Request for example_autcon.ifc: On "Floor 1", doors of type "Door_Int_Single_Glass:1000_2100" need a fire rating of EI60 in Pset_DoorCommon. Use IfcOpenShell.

First a look at what the model holds.

```python
import ifcopenshell
import ifcopenshell.util.element

model = ifcopenshell.open("example_autcon.ifc")
print(model.schema)
storey = next(s for s in model.by_type("IfcBuildingStorey") if s.Name == "Floor 1")
doors = [e for e in ifcopenshell.util.element.get_decomposition(storey) if e.is_a("IfcDoor")]
seen = {}
for e in doors:
    element_type = ifcopenshell.util.element.get_type(e)
    key = (element_type.Name if element_type != e and element_type else None, ifcopenshell.util.element.get_pset(e, "Pset_DoorCommon", "FireRating"))
    seen[key] = seen.get(key, 0) + 1
for (name, value), count in sorted(seen.items(), key=str):
    print(count, "x", name, "|", value)
```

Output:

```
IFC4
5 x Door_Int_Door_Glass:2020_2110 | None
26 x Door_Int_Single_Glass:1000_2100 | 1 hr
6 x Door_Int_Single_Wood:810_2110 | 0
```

```python
import ifcopenshell
import ifcopenshell.api.pset
import ifcopenshell.util.element

model = ifcopenshell.open("example_autcon.ifc")

storey = next(s for s in model.by_type("IfcBuildingStorey") if s.Name == "Floor 1")
doors = [e for e in ifcopenshell.util.element.get_decomposition(storey) if e.is_a("IfcDoor")]

count = 0
for e in doors:
    element_type = ifcopenshell.util.element.get_type(e)
    if element_type in (None, e) or element_type.Name != "Door_Int_Single_Glass:1000_2100":
        continue
    # add_pset returns the element's existing set when there is one.
    pset = ifcopenshell.api.pset.add_pset(model, product=e, name="Pset_DoorCommon")
    ifcopenshell.api.pset.edit_pset(model, pset=pset, properties={"FireRating": "EI60"})
    count += 1

print(count, "doors updated")

model.write("example_autcon_edited.ifc")
```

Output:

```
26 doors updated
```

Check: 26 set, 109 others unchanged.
